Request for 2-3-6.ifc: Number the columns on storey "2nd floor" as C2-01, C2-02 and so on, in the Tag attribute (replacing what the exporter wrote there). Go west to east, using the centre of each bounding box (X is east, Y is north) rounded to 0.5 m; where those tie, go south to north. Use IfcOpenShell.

First a look at what the model holds.

```python
import ifcopenshell
import ifcopenshell.util.element
import ifcopenshell.util.placement

model = ifcopenshell.open("2-3-6.ifc")
print(model.schema)
storey = next(s for s in model.by_type("IfcBuildingStorey") if s.Name == "2nd floor")
columns = [e for e in ifcopenshell.util.element.get_decomposition(storey) if e.is_a("IfcColumn")]
for e in sorted(columns, key=lambda e: e.id()):
    origin = ifcopenshell.util.placement.get_local_placement(e.ObjectPlacement)[:3, 3]
    print(e.id(), e.Tag, e.Name, origin.round(2) + 0.0, sep=" | ")
```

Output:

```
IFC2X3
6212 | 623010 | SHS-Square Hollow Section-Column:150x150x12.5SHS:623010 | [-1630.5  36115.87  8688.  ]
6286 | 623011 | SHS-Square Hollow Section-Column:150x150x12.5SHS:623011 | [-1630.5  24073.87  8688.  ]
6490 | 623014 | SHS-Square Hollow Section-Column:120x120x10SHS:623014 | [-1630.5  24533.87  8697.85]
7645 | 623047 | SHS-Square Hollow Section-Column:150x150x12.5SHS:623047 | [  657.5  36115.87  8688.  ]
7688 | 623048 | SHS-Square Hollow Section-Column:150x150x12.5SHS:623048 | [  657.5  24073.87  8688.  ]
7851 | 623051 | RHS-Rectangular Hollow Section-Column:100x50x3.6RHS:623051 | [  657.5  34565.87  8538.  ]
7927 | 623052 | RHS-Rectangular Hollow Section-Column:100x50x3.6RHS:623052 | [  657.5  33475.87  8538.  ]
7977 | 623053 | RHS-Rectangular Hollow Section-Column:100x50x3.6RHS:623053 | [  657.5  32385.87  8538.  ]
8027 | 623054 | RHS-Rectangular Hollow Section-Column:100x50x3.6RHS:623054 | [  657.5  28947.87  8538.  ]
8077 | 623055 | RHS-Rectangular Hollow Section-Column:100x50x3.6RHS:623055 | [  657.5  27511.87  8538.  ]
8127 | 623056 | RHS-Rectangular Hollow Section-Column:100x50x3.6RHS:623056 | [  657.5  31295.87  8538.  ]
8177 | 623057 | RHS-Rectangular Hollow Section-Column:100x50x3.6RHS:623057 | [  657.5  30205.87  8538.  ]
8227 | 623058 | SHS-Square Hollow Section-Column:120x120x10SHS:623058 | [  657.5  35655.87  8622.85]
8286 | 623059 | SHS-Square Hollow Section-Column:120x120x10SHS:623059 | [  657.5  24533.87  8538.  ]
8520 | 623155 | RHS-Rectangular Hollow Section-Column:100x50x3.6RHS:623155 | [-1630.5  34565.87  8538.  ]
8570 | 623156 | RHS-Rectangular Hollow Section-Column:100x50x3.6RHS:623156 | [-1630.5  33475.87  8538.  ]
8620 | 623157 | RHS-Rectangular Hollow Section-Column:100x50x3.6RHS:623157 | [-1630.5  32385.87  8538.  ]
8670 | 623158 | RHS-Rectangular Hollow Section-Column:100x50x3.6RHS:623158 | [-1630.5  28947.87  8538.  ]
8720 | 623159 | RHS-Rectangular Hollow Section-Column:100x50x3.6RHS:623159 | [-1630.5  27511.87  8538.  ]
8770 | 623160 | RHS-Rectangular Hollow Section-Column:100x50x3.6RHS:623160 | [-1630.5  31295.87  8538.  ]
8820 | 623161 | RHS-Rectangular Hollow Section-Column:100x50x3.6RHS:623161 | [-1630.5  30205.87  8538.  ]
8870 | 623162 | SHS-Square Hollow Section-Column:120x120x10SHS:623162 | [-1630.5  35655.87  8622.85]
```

```python
import ifcopenshell
import ifcopenshell.geom
import ifcopenshell.util.element
import ifcopenshell.util.shape

model = ifcopenshell.open("2-3-6.ifc")
settings = ifcopenshell.geom.settings()
settings.set("use-world-coords", True)


def centre(element):
    shape = ifcopenshell.geom.create_shape(settings, element)
    return ifcopenshell.util.shape.get_bbox_centroid(shape.geometry)


storey = next(s for s in model.by_type("IfcBuildingStorey") if s.Name == "2nd floor")
columns = [e for e in ifcopenshell.util.element.get_decomposition(storey) if e.is_a("IfcColumn")]

# Insertion points can sit at a corner or the storey origin, so sort by the geometry (in metres).
centres = {e: centre(e) for e in columns}
columns.sort(key=lambda e: (round(centres[e][0] / 0.5), centres[e][1]))

for i, e in enumerate(columns, start=1):
    number = f"C2-{i:02d}"
    e.Tag = number
    print(e.id(), number)

model.write("2-3-6_edited.ifc")
```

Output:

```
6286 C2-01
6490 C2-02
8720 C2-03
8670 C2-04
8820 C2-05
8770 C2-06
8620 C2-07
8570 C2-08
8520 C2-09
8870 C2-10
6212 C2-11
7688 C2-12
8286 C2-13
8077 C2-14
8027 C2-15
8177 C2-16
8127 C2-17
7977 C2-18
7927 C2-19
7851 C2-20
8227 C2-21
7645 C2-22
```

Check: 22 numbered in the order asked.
